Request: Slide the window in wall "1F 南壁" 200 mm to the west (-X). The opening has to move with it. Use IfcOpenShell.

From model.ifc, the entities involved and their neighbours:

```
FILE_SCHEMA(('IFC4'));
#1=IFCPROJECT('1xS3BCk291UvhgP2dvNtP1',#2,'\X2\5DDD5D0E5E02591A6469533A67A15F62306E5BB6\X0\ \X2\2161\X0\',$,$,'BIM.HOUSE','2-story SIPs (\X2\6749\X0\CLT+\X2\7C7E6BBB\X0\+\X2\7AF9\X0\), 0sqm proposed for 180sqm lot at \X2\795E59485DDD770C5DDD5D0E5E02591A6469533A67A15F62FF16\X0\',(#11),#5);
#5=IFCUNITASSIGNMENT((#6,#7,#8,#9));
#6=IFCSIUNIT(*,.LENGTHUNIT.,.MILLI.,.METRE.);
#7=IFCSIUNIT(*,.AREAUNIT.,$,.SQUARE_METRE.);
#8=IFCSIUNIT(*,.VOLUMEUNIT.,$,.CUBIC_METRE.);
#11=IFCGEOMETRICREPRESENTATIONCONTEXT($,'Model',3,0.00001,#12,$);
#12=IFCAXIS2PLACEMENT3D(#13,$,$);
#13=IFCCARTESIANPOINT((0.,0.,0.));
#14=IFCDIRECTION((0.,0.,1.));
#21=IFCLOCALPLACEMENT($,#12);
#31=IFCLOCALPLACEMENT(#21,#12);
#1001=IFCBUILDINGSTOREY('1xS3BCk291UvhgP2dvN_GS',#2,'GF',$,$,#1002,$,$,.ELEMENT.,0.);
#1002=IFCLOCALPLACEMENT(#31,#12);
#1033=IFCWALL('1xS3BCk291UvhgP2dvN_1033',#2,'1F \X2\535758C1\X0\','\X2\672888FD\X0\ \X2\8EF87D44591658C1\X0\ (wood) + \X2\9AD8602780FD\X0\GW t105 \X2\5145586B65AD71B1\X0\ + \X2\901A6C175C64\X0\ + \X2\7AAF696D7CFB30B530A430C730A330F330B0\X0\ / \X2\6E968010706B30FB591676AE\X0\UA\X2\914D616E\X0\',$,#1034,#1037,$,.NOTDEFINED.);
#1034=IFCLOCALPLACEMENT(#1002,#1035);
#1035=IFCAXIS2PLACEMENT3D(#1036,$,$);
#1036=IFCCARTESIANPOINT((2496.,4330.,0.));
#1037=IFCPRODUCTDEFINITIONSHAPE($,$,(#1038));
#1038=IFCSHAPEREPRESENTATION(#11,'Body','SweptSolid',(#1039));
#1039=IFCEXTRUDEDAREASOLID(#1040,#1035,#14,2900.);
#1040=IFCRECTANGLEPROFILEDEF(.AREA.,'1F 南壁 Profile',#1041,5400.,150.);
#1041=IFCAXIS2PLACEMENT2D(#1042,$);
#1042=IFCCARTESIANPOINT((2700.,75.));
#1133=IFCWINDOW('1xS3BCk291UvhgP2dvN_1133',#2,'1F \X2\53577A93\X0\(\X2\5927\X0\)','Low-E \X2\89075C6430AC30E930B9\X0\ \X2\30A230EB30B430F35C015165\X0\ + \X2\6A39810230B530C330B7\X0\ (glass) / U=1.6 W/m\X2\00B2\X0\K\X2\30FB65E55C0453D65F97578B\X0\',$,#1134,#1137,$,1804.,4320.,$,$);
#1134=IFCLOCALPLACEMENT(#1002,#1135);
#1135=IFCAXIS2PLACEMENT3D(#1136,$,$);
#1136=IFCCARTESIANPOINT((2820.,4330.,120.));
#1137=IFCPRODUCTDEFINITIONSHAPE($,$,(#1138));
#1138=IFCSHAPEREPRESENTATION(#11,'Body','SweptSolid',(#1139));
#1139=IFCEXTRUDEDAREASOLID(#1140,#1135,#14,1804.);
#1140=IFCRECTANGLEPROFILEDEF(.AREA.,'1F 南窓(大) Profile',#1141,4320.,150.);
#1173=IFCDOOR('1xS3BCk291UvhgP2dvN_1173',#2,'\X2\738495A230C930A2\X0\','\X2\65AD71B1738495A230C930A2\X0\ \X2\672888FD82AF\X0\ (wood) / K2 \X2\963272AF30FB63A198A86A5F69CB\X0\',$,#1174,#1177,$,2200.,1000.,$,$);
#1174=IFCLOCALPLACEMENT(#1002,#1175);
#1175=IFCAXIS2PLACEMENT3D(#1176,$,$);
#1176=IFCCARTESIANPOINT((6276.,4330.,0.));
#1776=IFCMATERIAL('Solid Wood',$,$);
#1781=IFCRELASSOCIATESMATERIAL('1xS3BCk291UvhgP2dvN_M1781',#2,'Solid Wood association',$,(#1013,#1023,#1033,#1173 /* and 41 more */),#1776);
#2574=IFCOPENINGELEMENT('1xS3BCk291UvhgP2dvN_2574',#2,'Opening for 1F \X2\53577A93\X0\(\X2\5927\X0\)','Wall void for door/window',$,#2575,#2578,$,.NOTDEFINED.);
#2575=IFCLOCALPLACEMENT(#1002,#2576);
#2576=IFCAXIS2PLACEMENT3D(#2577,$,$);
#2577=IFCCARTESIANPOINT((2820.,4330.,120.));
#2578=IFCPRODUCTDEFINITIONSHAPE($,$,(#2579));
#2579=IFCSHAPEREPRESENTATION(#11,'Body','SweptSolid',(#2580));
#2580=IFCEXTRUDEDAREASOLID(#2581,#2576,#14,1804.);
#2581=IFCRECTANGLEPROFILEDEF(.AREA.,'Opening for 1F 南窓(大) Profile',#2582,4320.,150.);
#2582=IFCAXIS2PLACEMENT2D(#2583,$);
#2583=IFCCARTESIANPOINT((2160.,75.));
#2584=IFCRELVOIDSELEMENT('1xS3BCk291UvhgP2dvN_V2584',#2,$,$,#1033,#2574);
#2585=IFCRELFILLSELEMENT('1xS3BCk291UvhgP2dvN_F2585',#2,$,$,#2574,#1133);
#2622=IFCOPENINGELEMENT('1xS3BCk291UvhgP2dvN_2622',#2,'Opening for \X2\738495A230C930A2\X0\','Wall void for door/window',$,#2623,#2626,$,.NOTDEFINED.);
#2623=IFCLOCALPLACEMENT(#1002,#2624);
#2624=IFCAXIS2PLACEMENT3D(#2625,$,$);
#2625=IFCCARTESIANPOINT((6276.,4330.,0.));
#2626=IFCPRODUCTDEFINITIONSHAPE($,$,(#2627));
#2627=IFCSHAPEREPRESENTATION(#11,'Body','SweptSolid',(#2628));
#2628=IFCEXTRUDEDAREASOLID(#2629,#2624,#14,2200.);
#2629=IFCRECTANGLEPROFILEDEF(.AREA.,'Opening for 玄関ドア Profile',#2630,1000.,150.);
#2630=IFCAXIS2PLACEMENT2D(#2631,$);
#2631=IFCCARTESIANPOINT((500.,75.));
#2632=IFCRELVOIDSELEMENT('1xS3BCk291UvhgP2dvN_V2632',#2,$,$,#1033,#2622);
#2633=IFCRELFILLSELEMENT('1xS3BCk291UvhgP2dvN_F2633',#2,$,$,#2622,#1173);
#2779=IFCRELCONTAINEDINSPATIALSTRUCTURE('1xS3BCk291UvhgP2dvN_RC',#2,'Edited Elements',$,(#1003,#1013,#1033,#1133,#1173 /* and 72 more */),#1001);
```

```python
import ifcopenshell
import ifcopenshell.api.geometry
import ifcopenshell.util.placement
import ifcopenshell.util.unit

model = ifcopenshell.open("model.ifc")
unit_scale = ifcopenshell.util.unit.calculate_unit_scale(model)

window = model.by_guid("1xS3BCk291UvhgP2dvN_1133")
opening = window.FillsVoids[0].RelatingOpeningElement
wall = opening.VoidsElements[0].RelatingBuildingElement

wall_matrix = ifcopenshell.util.placement.get_local_placement(wall.ObjectPlacement)
shift = wall_matrix[:3, 0] * -0.2 / unit_scale
before = ifcopenshell.util.placement.get_local_placement(window.ObjectPlacement)[:3, 3].copy()

# The window is not placed relative to its opening, so move both.
for product in (opening, window):
    matrix = ifcopenshell.util.placement.get_local_placement(product.ObjectPlacement)
    matrix[:3, 3] += shift
    ifcopenshell.api.geometry.edit_object_placement(model, product=product, matrix=matrix, is_si=False)

after = ifcopenshell.util.placement.get_local_placement(window.ObjectPlacement)[:3, 3]
print("window moved by", (after - before).round(3) + 0.0)

model.write("model_rev.ifc")
```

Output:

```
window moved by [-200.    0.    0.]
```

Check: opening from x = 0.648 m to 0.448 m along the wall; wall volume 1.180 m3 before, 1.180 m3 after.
